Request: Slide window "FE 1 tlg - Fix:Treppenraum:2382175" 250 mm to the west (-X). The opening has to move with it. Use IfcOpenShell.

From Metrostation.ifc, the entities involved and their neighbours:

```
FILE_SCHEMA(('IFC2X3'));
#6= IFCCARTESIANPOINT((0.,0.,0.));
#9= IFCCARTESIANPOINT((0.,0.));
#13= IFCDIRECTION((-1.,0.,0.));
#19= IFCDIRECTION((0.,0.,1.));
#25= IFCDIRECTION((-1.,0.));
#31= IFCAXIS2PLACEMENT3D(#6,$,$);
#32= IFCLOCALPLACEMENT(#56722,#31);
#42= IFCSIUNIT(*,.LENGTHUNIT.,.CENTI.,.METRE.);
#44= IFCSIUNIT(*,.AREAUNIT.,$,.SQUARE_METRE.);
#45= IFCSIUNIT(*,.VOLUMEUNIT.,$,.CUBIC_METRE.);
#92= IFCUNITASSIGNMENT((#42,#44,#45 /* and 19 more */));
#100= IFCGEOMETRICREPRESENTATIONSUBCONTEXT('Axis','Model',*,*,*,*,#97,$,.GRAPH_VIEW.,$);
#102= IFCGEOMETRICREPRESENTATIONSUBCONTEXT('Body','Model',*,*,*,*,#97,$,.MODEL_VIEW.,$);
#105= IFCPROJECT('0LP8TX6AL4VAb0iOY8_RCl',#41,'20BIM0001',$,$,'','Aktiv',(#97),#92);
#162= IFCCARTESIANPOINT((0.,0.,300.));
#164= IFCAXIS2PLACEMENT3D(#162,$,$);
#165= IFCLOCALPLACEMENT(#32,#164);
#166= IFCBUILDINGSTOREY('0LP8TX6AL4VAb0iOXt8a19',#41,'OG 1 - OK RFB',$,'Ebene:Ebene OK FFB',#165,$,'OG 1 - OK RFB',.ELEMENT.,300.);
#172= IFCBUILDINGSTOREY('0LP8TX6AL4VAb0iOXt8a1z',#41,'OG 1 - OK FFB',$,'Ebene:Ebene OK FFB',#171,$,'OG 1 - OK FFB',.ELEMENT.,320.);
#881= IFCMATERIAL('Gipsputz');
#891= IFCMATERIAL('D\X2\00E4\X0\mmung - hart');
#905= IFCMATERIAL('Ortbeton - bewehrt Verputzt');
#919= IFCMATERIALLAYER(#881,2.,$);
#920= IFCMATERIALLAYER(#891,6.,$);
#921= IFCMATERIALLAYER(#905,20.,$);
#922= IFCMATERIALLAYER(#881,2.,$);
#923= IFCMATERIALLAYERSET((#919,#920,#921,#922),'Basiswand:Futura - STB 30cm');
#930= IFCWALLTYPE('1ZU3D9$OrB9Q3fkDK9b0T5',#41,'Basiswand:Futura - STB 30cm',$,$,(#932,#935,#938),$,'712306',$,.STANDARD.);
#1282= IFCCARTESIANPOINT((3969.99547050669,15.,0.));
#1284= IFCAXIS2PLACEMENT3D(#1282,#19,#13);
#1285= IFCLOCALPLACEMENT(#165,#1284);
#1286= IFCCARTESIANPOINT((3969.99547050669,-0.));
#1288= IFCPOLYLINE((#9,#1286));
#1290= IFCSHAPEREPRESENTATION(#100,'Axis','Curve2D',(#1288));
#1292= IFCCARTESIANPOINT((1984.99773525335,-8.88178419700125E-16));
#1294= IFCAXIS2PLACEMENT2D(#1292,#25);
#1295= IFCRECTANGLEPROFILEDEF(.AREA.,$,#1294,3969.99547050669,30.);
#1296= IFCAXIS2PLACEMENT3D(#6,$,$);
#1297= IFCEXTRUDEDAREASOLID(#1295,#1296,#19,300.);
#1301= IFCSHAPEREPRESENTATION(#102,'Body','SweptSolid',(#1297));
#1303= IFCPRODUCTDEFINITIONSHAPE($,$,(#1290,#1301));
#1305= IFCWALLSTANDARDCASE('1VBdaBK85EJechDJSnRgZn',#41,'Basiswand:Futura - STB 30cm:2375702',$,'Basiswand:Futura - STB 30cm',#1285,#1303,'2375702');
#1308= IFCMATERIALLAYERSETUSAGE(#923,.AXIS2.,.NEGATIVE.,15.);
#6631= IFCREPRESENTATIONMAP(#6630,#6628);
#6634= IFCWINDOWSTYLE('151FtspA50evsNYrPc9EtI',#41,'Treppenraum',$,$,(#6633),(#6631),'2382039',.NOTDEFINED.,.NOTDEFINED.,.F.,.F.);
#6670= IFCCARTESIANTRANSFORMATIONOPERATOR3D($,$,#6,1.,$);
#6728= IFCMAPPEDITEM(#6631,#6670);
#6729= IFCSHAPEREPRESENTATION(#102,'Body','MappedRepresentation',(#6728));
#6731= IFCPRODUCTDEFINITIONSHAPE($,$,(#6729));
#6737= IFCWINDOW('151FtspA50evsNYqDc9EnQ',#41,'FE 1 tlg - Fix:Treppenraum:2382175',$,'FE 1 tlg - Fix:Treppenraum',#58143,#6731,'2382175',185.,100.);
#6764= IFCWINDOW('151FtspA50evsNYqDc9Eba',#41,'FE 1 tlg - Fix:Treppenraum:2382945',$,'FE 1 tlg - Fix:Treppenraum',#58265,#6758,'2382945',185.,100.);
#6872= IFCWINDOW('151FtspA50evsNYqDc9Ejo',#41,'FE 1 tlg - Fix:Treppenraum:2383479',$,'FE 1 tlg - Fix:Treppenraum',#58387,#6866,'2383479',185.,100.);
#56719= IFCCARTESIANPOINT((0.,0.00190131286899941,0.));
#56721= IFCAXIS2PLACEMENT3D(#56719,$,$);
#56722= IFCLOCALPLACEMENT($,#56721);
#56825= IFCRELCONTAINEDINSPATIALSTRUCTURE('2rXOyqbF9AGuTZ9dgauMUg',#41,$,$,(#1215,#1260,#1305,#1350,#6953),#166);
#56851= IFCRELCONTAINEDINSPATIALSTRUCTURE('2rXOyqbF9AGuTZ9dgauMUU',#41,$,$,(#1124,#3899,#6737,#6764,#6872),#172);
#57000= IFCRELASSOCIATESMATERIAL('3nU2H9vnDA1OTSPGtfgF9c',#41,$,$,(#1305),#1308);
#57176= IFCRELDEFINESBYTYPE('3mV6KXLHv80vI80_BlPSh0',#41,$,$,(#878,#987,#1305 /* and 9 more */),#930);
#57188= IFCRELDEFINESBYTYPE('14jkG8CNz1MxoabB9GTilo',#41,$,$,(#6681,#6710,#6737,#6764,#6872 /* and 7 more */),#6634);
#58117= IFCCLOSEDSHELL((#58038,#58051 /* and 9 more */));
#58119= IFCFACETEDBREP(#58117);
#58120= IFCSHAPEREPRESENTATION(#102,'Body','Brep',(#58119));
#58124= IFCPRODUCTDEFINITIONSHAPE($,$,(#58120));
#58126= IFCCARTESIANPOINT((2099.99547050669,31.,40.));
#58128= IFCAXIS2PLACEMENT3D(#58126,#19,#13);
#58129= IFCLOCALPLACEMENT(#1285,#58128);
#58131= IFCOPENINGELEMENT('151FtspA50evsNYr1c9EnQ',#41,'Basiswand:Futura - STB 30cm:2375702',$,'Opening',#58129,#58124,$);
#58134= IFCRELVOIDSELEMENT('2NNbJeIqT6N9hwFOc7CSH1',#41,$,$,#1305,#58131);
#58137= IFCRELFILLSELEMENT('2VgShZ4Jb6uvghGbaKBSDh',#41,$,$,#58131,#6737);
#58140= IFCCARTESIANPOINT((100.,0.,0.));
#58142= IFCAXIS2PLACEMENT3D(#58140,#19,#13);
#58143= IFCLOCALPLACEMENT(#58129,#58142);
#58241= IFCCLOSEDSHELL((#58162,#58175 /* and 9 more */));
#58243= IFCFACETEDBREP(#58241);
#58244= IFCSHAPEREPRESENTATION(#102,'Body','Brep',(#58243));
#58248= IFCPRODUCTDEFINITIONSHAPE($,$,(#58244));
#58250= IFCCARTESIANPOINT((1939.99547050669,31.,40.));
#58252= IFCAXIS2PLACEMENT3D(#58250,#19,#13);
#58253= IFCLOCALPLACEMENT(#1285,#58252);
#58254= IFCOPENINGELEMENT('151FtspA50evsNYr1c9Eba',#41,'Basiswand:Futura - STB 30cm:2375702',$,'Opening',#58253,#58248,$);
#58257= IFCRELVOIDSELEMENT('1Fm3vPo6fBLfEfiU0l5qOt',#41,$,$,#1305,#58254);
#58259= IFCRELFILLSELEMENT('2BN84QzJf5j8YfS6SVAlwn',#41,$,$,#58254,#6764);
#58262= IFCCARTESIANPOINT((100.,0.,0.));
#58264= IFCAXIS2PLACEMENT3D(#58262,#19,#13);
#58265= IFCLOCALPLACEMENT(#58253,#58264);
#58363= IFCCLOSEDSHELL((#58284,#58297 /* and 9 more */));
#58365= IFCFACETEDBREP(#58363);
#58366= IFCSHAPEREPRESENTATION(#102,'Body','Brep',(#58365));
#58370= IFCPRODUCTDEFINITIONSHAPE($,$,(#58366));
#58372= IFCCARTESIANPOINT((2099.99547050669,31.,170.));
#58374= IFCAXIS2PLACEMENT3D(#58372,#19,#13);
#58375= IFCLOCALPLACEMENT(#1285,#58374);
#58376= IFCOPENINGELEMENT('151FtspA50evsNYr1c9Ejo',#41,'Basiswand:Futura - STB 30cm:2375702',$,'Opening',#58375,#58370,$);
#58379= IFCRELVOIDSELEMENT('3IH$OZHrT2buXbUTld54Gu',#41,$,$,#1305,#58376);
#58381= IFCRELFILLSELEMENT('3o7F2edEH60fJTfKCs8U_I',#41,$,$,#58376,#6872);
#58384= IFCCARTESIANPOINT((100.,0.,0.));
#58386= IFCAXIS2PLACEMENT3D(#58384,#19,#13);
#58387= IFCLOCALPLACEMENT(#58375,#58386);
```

```python
import ifcopenshell
import ifcopenshell.api.geometry
import ifcopenshell.util.placement
import ifcopenshell.util.unit

model = ifcopenshell.open("Metrostation.ifc")
unit_scale = ifcopenshell.util.unit.calculate_unit_scale(model)

window = model.by_guid("151FtspA50evsNYqDc9EnQ")
opening = window.FillsVoids[0].RelatingOpeningElement
wall = opening.VoidsElements[0].RelatingBuildingElement

wall_matrix = ifcopenshell.util.placement.get_local_placement(wall.ObjectPlacement)
shift = wall_matrix[:3, 0] * 0.25 / unit_scale
before = ifcopenshell.util.placement.get_local_placement(window.ObjectPlacement)[:3, 3].copy()

# The window is placed relative to its opening, so it follows when the opening moves.
matrix = ifcopenshell.util.placement.get_local_placement(opening.ObjectPlacement)
matrix[:3, 3] += shift
ifcopenshell.api.geometry.edit_object_placement(
    model, product=opening, matrix=matrix, is_si=False, should_transform_children=True
)

after = ifcopenshell.util.placement.get_local_placement(window.ObjectPlacement)[:3, 3]
print("window moved by", (after - before).round(3) + 0.0)

model.write("Metrostation_edited.ifc")
```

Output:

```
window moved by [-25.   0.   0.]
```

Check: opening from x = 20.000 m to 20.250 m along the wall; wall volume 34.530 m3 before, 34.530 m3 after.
